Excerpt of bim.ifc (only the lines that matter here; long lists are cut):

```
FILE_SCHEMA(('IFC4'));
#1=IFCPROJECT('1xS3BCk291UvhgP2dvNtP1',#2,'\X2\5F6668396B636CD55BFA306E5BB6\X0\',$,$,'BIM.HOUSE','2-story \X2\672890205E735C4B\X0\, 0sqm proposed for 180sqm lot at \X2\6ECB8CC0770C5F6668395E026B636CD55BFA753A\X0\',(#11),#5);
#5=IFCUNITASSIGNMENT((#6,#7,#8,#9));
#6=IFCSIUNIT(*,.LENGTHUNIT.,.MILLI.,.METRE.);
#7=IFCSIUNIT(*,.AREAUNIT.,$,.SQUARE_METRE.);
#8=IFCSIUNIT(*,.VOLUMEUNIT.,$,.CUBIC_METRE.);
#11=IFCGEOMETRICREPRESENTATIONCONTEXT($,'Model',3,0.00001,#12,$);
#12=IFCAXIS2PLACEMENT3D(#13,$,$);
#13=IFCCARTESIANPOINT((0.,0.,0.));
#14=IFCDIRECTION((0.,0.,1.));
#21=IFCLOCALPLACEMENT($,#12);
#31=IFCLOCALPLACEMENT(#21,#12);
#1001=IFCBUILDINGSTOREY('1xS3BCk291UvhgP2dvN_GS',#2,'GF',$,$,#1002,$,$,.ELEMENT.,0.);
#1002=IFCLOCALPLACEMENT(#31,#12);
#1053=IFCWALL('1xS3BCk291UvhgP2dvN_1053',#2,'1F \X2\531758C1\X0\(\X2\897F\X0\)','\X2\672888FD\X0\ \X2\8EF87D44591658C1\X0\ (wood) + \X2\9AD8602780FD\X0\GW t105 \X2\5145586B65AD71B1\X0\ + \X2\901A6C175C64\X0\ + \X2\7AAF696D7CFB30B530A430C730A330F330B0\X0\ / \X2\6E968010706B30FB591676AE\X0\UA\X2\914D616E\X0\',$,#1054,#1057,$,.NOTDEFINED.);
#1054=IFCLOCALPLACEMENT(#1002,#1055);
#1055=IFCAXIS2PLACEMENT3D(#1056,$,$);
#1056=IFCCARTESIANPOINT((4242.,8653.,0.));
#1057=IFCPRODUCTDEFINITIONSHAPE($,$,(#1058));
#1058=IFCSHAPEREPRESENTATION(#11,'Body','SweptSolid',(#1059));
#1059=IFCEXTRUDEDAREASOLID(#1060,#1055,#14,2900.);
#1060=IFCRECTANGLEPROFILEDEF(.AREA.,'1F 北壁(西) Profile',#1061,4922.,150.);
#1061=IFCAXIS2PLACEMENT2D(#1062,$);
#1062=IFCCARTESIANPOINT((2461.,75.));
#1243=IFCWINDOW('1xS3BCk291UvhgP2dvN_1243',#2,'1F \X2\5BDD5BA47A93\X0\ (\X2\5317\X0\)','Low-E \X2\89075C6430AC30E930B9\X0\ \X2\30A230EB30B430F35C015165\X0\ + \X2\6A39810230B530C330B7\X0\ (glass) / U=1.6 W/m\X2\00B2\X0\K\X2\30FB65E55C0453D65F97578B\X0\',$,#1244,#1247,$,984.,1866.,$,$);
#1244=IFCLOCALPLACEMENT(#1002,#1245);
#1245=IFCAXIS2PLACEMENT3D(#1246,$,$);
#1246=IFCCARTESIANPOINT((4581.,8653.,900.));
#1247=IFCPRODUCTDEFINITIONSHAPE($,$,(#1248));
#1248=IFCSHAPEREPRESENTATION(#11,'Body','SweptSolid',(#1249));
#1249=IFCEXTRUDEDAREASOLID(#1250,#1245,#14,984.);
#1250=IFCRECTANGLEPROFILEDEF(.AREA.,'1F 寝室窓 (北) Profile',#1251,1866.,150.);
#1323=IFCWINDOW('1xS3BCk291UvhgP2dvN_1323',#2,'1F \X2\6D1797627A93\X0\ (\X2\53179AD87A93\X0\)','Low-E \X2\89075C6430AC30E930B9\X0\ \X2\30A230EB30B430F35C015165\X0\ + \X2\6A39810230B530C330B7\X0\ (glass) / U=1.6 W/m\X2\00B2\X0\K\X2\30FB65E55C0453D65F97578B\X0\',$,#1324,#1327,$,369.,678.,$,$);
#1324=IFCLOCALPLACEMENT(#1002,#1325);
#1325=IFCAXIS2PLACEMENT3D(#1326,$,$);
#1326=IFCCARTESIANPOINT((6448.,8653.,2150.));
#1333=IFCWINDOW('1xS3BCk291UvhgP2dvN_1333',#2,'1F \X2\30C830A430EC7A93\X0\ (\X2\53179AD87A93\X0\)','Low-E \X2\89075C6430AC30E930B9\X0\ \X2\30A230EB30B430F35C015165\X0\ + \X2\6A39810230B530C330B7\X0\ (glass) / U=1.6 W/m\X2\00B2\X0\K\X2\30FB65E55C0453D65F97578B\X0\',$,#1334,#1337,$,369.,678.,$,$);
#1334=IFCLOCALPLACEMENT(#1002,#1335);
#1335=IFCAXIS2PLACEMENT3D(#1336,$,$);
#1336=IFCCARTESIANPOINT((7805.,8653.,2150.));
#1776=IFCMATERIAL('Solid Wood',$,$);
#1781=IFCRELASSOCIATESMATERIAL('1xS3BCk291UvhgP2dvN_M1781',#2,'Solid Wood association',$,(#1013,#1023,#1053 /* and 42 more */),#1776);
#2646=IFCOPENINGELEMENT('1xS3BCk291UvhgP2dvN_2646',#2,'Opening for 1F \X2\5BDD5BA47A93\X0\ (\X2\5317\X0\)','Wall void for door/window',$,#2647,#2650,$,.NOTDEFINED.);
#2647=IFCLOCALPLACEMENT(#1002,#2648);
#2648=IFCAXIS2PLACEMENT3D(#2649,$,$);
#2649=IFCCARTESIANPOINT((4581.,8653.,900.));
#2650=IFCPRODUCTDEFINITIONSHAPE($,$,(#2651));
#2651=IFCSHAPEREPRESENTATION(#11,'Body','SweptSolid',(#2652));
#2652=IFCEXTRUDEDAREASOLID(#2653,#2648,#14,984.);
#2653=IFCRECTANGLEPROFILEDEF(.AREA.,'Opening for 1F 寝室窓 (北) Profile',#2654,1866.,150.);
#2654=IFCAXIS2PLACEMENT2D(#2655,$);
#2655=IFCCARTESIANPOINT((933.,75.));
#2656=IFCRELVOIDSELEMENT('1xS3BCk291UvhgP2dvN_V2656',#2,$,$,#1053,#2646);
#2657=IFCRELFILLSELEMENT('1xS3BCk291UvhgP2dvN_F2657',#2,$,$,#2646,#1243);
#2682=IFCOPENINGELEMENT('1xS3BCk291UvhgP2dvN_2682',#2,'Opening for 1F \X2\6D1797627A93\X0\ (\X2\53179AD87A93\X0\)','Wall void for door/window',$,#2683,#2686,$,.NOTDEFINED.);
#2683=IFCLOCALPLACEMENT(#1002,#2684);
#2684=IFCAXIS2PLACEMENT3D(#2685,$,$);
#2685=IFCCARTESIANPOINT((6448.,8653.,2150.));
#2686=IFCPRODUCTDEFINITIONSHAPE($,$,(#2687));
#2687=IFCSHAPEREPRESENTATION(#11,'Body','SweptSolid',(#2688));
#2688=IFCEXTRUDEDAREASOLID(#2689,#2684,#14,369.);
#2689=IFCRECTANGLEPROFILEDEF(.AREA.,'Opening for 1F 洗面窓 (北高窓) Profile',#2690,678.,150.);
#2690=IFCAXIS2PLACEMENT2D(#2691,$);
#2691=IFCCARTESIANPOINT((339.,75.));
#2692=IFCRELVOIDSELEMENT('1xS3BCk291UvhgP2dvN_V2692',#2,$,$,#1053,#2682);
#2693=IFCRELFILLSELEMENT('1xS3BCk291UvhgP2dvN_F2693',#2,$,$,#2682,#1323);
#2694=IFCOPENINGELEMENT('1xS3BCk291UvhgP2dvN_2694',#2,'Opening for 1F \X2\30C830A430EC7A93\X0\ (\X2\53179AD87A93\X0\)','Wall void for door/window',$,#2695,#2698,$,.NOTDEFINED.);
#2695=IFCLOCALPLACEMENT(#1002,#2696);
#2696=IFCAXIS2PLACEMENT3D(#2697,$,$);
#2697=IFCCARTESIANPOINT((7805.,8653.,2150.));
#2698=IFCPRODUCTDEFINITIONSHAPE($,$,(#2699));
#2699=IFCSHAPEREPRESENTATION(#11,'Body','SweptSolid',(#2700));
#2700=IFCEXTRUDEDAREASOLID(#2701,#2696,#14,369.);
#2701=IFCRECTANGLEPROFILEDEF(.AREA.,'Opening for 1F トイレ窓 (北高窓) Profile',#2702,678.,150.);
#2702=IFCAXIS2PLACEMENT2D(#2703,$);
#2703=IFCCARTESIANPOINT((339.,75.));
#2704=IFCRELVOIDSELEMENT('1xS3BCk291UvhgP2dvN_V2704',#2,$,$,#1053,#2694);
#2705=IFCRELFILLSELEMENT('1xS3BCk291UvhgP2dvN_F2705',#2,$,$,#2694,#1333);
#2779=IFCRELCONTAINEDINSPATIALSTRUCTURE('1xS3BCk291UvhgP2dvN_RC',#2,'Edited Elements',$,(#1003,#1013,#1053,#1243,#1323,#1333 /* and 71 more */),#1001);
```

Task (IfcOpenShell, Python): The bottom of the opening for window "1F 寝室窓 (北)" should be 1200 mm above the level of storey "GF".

```python
import numpy as np
import ifcopenshell
import ifcopenshell.api.geometry
import ifcopenshell.geom
import ifcopenshell.util.element
import ifcopenshell.util.placement
import ifcopenshell.util.shape
import ifcopenshell.util.unit

model = ifcopenshell.open("bim.ifc")
unit_scale = ifcopenshell.util.unit.calculate_unit_scale(model)

window = model.by_id(1243)
opening = window.FillsVoids[0].RelatingOpeningElement
storey = ifcopenshell.util.element.get_container(window, ifc_class="IfcBuildingStorey")
level = ifcopenshell.util.placement.get_local_placement(storey.ObjectPlacement)[2, 3]

# The opening's origin need not be at the sill, so measure its lowest point.
shape = ifcopenshell.geom.create_shape(ifcopenshell.geom.settings(), opening)
bottom = ifcopenshell.util.shape.get_shape_bottom_elevation(shape, shape.geometry) / unit_scale
dz = level + 1.2 / unit_scale - bottom

shift = np.array([0.0, 0.0, dz])
# The window is not placed relative to its opening, so move both.
for product in (opening, window):
    matrix = ifcopenshell.util.placement.get_local_placement(product.ObjectPlacement)
    matrix[:3, 3] += shift
    ifcopenshell.api.geometry.edit_object_placement(model, product=product, matrix=matrix, is_si=False)

print(f"moved by {dz * unit_scale:+.3f} m")

model.write("bim_updated.ifc")
```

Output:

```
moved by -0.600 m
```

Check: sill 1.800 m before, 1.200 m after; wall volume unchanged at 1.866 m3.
